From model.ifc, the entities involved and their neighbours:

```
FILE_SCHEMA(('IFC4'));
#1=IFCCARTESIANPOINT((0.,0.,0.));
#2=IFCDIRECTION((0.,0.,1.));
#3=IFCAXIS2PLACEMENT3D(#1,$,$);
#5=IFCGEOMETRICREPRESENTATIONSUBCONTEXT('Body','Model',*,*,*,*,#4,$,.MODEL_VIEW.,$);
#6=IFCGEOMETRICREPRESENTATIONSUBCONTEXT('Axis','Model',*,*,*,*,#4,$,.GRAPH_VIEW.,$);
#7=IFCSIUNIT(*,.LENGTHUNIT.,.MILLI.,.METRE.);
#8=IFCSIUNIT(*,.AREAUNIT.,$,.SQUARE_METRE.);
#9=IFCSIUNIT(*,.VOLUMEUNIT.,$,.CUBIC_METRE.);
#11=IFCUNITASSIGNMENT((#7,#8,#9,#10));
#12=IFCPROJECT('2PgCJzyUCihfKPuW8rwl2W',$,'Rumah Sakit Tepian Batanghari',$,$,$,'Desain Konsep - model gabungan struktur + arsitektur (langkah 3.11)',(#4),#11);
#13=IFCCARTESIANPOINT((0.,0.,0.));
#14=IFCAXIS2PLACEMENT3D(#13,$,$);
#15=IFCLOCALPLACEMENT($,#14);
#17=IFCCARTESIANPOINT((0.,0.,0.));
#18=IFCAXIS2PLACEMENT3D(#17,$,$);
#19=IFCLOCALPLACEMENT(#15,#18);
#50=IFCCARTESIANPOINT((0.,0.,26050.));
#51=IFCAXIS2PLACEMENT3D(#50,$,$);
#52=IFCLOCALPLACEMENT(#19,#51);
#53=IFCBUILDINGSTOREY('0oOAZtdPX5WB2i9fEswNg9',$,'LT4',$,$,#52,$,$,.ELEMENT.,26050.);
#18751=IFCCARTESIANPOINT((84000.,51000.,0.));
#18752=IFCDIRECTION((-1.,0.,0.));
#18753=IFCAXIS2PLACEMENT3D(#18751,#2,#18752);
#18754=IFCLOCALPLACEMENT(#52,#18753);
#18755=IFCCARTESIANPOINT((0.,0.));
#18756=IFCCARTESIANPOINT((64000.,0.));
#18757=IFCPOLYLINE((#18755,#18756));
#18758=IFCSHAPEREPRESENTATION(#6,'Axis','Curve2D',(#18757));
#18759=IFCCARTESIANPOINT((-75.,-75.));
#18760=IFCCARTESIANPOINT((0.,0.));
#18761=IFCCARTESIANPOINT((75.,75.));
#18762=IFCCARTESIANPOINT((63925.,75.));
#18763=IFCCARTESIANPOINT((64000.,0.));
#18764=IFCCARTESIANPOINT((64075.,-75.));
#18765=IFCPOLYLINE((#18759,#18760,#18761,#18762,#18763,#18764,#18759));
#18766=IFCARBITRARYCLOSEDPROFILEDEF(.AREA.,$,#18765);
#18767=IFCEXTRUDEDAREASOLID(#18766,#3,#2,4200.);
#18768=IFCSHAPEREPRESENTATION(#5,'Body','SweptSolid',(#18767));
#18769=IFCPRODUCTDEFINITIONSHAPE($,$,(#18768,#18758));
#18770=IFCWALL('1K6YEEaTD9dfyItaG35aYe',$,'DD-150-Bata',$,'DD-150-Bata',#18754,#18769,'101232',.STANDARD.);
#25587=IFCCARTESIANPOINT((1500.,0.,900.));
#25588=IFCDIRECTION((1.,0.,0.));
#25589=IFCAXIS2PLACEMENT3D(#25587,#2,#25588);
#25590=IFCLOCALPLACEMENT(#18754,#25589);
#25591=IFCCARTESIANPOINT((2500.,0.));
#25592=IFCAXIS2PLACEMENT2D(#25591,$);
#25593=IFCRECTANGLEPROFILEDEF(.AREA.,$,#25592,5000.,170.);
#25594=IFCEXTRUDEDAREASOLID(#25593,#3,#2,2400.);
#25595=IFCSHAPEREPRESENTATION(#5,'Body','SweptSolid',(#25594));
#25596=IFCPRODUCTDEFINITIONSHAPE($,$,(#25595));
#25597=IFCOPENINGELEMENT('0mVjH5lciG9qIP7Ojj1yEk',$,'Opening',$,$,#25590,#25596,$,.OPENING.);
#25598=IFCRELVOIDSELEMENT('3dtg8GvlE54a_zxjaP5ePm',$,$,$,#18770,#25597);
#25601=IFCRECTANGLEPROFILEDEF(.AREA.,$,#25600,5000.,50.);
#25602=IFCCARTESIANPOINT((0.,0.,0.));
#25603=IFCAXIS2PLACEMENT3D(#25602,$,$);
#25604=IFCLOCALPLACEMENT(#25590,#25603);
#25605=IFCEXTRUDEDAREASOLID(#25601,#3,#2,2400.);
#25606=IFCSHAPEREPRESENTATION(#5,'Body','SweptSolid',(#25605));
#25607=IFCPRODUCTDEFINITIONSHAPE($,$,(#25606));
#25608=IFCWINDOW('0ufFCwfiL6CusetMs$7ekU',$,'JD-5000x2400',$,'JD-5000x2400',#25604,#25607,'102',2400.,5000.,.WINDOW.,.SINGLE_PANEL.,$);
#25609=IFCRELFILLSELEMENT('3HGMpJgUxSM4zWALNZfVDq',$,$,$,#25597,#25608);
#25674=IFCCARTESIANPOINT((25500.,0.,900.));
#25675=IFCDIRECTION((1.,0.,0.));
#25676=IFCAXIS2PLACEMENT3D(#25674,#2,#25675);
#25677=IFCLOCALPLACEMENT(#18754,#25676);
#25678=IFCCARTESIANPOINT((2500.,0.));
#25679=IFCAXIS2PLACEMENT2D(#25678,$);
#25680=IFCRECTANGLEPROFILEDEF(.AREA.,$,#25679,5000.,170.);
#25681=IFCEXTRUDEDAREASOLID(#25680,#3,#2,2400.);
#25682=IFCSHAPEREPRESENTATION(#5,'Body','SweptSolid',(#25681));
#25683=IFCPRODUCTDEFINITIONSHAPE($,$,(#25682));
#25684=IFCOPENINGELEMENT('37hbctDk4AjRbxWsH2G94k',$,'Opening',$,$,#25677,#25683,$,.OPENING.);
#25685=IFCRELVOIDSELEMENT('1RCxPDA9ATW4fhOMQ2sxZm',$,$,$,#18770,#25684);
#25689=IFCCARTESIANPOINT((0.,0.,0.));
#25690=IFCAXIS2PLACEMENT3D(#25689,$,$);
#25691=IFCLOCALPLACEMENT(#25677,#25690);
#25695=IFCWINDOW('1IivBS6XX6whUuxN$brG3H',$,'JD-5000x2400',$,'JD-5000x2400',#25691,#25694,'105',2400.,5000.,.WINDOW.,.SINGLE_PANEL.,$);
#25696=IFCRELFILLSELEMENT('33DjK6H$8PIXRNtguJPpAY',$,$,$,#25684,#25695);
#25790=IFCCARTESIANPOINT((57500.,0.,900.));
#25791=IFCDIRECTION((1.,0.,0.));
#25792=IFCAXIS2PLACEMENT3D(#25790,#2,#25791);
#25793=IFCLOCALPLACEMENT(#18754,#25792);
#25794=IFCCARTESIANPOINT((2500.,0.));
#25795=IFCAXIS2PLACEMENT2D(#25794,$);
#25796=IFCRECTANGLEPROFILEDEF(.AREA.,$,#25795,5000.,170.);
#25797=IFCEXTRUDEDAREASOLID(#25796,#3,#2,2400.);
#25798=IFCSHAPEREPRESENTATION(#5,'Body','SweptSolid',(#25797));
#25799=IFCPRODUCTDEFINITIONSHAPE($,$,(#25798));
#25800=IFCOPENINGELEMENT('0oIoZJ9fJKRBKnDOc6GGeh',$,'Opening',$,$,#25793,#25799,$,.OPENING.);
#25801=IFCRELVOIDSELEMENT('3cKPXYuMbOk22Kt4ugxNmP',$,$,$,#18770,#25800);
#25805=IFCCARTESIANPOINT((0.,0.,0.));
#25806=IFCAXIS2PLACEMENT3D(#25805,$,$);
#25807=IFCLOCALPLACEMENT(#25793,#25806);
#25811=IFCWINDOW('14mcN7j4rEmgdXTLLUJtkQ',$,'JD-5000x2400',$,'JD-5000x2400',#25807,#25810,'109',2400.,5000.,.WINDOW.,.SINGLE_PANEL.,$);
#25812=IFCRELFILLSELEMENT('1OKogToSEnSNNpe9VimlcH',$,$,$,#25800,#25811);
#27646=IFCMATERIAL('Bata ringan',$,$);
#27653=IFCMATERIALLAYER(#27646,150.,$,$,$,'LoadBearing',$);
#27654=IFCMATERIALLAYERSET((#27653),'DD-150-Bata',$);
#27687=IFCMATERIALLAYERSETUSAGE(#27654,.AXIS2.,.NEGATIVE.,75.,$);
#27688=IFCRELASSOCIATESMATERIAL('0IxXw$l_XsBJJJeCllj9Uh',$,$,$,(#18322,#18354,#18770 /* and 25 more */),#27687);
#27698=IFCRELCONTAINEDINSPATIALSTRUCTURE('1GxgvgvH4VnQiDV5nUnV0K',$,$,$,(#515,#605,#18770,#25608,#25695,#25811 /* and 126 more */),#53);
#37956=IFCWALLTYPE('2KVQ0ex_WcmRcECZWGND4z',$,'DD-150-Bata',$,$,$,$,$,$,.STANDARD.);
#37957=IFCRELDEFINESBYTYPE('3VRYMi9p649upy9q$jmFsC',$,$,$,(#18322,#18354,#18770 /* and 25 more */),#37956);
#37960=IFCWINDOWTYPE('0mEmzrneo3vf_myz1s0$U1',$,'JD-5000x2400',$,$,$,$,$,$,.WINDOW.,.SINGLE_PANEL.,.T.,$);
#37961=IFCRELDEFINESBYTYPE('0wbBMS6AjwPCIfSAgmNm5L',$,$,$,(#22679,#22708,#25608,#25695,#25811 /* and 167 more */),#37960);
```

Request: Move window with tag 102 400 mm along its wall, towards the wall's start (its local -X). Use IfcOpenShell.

```python
import ifcopenshell
import ifcopenshell.api.geometry
import ifcopenshell.util.placement
import ifcopenshell.util.unit

model = ifcopenshell.open("model.ifc")
unit_scale = ifcopenshell.util.unit.calculate_unit_scale(model)

window = model.by_id(25608)
opening = window.FillsVoids[0].RelatingOpeningElement
wall = opening.VoidsElements[0].RelatingBuildingElement

wall_matrix = ifcopenshell.util.placement.get_local_placement(wall.ObjectPlacement)
shift = wall_matrix[:3, 0] * -0.4 / unit_scale
before = ifcopenshell.util.placement.get_local_placement(window.ObjectPlacement)[:3, 3].copy()

# The window is placed relative to its opening, so it follows when the opening moves.
matrix = ifcopenshell.util.placement.get_local_placement(opening.ObjectPlacement)
matrix[:3, 3] += shift
ifcopenshell.api.geometry.edit_object_placement(
    model, product=opening, matrix=matrix, is_si=False, should_transform_children=True
)

after = ifcopenshell.util.placement.get_local_placement(window.ObjectPlacement)[:3, 3]
print("window moved by", (after - before).round(3) + 0.0)

model.write("model_rev.ifc")
```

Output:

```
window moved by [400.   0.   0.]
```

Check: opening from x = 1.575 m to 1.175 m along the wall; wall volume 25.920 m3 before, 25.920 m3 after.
